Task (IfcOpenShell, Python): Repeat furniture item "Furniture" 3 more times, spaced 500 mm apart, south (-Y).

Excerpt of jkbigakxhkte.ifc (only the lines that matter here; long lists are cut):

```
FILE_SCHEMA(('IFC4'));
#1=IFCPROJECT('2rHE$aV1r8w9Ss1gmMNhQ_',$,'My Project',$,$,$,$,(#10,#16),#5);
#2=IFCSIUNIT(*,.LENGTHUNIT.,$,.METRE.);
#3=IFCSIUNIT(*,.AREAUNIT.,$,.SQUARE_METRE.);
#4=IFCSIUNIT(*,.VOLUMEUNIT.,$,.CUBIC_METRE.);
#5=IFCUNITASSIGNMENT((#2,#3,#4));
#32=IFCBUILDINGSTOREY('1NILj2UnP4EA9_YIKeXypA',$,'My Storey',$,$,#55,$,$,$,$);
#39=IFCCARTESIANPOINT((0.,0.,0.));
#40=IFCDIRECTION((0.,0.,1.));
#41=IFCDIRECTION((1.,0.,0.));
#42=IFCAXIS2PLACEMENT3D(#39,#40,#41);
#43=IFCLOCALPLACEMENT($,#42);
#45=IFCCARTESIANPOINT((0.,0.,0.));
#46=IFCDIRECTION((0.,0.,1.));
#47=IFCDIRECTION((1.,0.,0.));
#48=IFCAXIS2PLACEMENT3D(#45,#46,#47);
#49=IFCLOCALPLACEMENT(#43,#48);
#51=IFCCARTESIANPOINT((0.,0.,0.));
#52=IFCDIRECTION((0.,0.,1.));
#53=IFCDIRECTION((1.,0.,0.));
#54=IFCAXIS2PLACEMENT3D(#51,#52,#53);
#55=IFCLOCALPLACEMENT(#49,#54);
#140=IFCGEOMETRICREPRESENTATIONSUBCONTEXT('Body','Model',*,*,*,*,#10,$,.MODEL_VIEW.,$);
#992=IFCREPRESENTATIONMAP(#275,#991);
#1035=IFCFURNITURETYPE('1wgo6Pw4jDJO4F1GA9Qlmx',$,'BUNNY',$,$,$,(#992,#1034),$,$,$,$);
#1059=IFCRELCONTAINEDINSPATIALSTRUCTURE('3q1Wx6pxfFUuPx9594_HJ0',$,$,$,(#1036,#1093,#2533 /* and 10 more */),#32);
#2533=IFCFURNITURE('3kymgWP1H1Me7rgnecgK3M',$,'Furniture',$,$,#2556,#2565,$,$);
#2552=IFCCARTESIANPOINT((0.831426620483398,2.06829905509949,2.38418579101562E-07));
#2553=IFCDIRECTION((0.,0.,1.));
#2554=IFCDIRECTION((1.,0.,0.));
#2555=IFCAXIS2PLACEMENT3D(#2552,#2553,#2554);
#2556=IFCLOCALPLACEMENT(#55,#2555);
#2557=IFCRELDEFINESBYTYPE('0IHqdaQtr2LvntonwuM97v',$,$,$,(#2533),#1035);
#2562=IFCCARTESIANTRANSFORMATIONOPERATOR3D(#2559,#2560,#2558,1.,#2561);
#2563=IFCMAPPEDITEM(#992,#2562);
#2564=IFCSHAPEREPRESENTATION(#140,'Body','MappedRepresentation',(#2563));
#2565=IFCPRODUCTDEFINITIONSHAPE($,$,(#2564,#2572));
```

```python
import numpy as np
import ifcopenshell
import ifcopenshell.api.geometry
import ifcopenshell.api.root
import ifcopenshell.util.element
import ifcopenshell.util.placement
import ifcopenshell.util.unit

model = ifcopenshell.open("jkbigakxhkte.ifc")
unit_scale = ifcopenshell.util.unit.calculate_unit_scale(model)

source = model.by_guid("3kymgWP1H1Me7rgnecgK3M")
base = ifcopenshell.util.placement.get_local_placement(source.ObjectPlacement)
step = np.array([0.0, -1.0, 0.0]) * 0.5 / unit_scale

for i in range(1, 4):
    copy = ifcopenshell.api.root.copy_class(model, product=source)
    copy.Representation = ifcopenshell.util.element.copy_deep(
        model, source.Representation, exclude=["IfcGeometricRepresentationContext", "IfcRepresentationMap"]
    )
    matrix = base.copy()
    matrix[:3, 3] += i * step
    print("added at", matrix[:3, 3].round(3) + 0.0)
    ifcopenshell.api.geometry.edit_object_placement(model, product=copy, matrix=matrix, is_si=False)

model.write("jkbigakxhkte-out.ifc")
```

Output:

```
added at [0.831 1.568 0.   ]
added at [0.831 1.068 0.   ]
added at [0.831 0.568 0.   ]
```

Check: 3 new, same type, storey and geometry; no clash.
